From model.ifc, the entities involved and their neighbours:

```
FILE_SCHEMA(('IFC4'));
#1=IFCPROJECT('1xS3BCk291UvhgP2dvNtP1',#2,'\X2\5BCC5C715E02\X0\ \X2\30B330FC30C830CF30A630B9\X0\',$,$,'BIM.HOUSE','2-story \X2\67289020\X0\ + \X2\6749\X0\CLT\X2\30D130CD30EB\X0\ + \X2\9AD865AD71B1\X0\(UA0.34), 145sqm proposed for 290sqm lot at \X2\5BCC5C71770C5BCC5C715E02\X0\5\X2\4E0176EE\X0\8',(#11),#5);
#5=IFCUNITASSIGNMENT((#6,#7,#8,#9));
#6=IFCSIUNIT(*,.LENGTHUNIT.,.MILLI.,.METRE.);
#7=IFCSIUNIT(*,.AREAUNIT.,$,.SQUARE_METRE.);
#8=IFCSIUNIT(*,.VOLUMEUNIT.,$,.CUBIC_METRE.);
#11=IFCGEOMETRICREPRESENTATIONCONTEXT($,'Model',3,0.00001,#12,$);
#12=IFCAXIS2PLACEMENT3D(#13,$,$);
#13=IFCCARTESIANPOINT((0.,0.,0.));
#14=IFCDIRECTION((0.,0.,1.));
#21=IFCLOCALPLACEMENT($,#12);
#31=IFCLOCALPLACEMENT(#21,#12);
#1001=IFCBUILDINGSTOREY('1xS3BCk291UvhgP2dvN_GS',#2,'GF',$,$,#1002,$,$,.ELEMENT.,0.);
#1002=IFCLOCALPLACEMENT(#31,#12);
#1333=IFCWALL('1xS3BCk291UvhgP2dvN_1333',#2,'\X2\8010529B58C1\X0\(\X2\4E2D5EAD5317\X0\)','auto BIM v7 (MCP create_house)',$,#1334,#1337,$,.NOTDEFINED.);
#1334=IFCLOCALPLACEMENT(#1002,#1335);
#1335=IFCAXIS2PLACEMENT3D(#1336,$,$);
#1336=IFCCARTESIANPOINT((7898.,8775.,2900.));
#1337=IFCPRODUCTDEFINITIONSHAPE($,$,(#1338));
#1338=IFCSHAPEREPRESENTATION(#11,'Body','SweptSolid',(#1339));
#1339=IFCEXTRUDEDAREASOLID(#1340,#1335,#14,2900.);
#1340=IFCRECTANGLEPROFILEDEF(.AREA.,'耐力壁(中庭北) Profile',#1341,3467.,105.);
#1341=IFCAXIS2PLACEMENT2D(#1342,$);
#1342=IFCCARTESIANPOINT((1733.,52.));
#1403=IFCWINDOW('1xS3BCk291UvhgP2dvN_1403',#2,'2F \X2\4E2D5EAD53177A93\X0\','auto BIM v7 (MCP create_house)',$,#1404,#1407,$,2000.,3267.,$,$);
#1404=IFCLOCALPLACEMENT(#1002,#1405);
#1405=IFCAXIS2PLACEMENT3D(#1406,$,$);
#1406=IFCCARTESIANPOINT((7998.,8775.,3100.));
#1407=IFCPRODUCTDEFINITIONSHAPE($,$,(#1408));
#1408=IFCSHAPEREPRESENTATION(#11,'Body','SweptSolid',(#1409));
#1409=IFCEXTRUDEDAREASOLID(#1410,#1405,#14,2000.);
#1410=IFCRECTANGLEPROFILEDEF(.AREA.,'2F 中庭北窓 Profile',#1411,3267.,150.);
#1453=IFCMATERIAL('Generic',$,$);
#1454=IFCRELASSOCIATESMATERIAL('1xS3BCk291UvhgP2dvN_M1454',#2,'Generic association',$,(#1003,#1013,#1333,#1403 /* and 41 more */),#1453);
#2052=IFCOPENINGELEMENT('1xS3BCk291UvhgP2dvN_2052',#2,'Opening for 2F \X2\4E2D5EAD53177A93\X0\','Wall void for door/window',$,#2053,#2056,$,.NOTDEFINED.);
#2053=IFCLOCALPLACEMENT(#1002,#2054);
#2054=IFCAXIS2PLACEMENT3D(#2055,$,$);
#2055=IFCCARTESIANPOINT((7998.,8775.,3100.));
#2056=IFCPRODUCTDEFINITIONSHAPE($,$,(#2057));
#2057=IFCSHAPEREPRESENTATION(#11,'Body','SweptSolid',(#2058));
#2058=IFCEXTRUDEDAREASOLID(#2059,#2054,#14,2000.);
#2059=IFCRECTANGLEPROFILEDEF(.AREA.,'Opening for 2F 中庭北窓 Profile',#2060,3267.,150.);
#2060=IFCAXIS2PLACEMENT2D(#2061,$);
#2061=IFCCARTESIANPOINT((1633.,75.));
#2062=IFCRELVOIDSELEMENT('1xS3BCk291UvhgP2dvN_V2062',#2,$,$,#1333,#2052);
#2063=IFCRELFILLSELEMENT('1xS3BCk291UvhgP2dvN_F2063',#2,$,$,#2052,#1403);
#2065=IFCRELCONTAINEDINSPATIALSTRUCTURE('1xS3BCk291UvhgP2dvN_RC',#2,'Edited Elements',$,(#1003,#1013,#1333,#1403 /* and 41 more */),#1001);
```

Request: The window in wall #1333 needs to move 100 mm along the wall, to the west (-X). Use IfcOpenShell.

```python
import ifcopenshell
import ifcopenshell.api.geometry
import ifcopenshell.util.placement
import ifcopenshell.util.unit

model = ifcopenshell.open("model.ifc")
unit_scale = ifcopenshell.util.unit.calculate_unit_scale(model)

window = model.by_guid("1xS3BCk291UvhgP2dvN_1403")
opening = window.FillsVoids[0].RelatingOpeningElement
wall = opening.VoidsElements[0].RelatingBuildingElement

wall_matrix = ifcopenshell.util.placement.get_local_placement(wall.ObjectPlacement)
shift = wall_matrix[:3, 0] * -0.1 / unit_scale
before = ifcopenshell.util.placement.get_local_placement(window.ObjectPlacement)[:3, 3].copy()

# The window is not placed relative to its opening, so move both.
for product in (opening, window):
    matrix = ifcopenshell.util.placement.get_local_placement(product.ObjectPlacement)
    matrix[:3, 3] += shift
    ifcopenshell.api.geometry.edit_object_placement(model, product=product, matrix=matrix, is_si=False)

after = ifcopenshell.util.placement.get_local_placement(window.ObjectPlacement)[:3, 3]
print("window moved by", (after - before).round(3) + 0.0)

model.write("model_edited.ifc")
```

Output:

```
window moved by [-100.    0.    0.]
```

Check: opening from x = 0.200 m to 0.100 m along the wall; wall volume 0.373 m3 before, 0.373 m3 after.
